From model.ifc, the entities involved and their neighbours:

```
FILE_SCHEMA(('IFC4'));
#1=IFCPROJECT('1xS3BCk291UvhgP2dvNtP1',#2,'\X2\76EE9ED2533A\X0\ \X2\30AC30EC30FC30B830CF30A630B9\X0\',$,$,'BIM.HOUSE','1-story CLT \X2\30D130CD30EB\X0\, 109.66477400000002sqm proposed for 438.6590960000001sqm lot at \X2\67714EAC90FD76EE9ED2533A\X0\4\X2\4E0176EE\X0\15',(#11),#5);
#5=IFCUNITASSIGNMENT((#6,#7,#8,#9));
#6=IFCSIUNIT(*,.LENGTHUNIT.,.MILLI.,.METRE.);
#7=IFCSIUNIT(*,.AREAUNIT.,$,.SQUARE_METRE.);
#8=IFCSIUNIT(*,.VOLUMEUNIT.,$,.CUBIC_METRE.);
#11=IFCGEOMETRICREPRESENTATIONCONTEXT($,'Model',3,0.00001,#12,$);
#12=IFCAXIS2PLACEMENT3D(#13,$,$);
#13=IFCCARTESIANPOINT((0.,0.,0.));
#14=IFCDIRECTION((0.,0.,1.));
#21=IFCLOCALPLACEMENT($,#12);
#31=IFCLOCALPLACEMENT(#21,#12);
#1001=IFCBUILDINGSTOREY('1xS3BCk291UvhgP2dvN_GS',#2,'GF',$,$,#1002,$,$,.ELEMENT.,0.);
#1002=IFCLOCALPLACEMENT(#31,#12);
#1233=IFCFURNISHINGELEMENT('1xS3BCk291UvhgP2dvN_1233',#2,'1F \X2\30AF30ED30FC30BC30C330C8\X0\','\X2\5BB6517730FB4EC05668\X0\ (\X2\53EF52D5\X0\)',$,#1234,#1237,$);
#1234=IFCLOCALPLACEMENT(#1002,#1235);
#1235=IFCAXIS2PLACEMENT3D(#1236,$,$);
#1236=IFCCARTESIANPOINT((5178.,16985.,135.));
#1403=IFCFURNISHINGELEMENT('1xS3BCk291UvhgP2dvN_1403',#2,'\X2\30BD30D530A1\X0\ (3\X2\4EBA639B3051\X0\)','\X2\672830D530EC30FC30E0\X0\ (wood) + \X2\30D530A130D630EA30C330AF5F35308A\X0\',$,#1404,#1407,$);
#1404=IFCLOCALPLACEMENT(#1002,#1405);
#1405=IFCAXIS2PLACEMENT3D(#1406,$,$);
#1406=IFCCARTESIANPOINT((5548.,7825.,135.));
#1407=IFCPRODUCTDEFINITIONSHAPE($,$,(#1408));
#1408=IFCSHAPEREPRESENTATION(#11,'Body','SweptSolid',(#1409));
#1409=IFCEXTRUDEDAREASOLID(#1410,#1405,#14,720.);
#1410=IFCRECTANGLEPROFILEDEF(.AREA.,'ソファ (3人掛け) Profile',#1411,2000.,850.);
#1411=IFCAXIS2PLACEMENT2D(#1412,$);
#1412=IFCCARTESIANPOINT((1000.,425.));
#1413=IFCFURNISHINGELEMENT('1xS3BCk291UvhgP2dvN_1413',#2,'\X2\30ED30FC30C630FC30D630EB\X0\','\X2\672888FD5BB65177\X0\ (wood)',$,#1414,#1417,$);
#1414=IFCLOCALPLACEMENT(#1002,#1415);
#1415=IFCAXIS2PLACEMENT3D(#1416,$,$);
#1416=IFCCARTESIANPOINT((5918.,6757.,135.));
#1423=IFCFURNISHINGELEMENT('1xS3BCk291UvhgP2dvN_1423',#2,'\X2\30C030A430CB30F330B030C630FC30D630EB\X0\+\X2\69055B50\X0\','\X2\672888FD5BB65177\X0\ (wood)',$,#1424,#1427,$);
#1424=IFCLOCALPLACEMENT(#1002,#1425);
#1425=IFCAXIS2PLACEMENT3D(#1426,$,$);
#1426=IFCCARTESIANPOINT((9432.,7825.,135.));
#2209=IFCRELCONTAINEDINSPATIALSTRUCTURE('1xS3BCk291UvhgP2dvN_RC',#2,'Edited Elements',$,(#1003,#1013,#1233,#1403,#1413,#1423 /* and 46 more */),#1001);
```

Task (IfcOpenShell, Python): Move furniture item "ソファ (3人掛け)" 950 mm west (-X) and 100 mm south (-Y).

```python
import ifcopenshell
import ifcopenshell.api.geometry
import ifcopenshell.util.placement
import ifcopenshell.util.unit

model = ifcopenshell.open("model.ifc")
unit_scale = ifcopenshell.util.unit.calculate_unit_scale(model)

item = model.by_id(1403)
matrix = ifcopenshell.util.placement.get_local_placement(item.ObjectPlacement)
matrix[0, 3] -= 0.95 / unit_scale
matrix[1, 3] -= 0.1 / unit_scale
ifcopenshell.api.geometry.edit_object_placement(model, product=item, matrix=matrix, is_si=False)

print(ifcopenshell.util.placement.get_local_placement(item.ObjectPlacement).round(3) + 0.0)

model.write("model-out.ifc")
```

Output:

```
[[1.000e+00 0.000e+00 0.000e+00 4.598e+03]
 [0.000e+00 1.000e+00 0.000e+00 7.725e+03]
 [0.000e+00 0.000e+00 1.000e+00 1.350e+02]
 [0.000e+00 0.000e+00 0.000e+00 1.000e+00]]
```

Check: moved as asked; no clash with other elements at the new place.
